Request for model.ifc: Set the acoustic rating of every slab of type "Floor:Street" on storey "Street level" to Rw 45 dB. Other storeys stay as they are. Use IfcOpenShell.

First a look at what the model holds.

```python
import ifcopenshell
import ifcopenshell.util.element

model = ifcopenshell.open("model.ifc")
print(model.schema)
storey = next(s for s in model.by_type("IfcBuildingStorey") if s.Name == "Street level")
slabs = [e for e in ifcopenshell.util.element.get_decomposition(storey) if e.is_a("IfcSlab")]
seen = {}
for e in slabs:
    element_type = ifcopenshell.util.element.get_type(e)
    key = (element_type.Name if element_type != e and element_type else None, ifcopenshell.util.element.get_pset(e, "Pset_SlabCommon", "AcousticRating"))
    seen[key] = seen.get(key, 0) + 1
for (name, value), count in sorted(seen.items(), key=str):
    print(count, "x", name, "|", value)
```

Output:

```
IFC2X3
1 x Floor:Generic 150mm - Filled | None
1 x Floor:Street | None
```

```python
import ifcopenshell
import ifcopenshell.api.pset
import ifcopenshell.util.element

model = ifcopenshell.open("model.ifc")

storey = next(s for s in model.by_type("IfcBuildingStorey") if s.Name == "Street level")
slabs = [e for e in ifcopenshell.util.element.get_decomposition(storey) if e.is_a("IfcSlab")]

count = 0
for e in slabs:
    element_type = ifcopenshell.util.element.get_type(e)
    if element_type in (None, e) or element_type.Name != "Floor:Street":
        continue
    # add_pset returns the element's existing set when there is one.
    pset = ifcopenshell.api.pset.add_pset(model, product=e, name="Pset_SlabCommon")
    ifcopenshell.api.pset.edit_pset(model, pset=pset, properties={"AcousticRating": "Rw 45 dB"})
    count += 1

print(count, "slabs updated")

model.write("model_edited.ifc")
```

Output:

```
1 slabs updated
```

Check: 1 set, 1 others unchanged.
